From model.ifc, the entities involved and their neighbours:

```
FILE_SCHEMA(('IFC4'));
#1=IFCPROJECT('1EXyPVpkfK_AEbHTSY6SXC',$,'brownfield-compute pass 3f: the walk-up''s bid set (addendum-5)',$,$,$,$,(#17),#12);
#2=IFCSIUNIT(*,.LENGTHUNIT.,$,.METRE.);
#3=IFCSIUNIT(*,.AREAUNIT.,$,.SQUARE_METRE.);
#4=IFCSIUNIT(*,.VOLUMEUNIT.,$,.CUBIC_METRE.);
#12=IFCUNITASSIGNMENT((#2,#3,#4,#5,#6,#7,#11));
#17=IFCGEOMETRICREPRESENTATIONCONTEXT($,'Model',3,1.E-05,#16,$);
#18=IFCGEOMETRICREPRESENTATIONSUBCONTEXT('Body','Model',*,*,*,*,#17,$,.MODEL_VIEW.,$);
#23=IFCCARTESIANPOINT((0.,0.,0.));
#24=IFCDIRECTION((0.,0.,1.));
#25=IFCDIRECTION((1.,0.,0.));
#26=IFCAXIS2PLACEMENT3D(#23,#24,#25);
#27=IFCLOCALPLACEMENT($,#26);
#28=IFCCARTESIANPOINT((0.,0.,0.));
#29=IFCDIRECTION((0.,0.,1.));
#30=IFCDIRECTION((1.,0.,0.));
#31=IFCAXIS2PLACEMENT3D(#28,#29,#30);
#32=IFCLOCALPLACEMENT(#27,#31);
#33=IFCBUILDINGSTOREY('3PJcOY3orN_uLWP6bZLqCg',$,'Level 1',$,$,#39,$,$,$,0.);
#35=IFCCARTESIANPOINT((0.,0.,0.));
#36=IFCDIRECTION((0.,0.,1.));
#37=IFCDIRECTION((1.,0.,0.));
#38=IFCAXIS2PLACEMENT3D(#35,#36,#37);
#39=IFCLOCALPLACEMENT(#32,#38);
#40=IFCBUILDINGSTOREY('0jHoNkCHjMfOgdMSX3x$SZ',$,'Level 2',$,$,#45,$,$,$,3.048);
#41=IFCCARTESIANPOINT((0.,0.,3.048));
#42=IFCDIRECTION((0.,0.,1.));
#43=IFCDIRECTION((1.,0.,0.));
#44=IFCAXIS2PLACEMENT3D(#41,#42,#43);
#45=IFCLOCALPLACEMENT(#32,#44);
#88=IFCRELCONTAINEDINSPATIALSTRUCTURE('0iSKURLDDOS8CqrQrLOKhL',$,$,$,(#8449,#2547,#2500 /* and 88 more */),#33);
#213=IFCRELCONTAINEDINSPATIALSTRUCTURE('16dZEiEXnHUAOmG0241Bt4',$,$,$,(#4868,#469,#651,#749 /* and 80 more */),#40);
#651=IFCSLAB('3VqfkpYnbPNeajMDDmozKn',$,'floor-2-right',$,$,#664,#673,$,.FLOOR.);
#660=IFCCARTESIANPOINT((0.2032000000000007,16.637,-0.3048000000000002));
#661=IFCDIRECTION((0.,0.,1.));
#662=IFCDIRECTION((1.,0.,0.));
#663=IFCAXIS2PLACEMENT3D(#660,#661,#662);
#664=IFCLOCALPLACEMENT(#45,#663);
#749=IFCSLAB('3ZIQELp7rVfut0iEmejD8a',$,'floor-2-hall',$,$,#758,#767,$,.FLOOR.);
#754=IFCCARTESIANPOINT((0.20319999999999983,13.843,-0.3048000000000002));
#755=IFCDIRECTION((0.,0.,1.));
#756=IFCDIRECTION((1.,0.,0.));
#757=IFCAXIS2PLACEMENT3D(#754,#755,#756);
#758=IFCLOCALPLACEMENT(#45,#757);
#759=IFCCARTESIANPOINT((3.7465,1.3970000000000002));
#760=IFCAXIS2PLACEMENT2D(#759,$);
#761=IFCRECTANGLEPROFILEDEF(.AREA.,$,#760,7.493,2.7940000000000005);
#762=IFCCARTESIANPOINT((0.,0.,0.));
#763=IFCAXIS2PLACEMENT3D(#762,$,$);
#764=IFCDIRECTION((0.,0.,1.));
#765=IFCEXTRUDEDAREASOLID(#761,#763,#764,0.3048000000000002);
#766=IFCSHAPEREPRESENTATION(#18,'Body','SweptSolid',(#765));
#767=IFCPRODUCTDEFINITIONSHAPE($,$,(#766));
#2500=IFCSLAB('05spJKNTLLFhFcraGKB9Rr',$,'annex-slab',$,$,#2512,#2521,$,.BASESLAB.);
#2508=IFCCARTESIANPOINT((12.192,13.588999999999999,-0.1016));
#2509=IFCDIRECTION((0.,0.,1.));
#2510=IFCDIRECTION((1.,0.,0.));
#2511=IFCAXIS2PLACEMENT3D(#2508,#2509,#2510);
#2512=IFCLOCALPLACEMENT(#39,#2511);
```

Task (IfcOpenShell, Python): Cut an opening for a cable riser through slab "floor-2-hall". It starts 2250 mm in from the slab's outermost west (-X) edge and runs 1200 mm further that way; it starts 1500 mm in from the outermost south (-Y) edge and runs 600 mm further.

```python
import numpy as np
import ifcopenshell
import ifcopenshell.api.feature
import ifcopenshell.api.geometry
import ifcopenshell.api.root
import ifcopenshell.geom
import ifcopenshell.util.placement
import ifcopenshell.util.representation
import ifcopenshell.util.shape
import ifcopenshell.util.unit

model = ifcopenshell.open("model.ifc")
unit_scale = ifcopenshell.util.unit.calculate_unit_scale(model)
settings = ifcopenshell.geom.settings()


def volume(element):
    """Net volume in cubic metres, openings subtracted."""
    shape = ifcopenshell.geom.create_shape(settings, element)
    return ifcopenshell.util.shape.get_volume(shape.geometry)


slab = model.by_guid("3ZIQELp7rVfut0iEmejD8a")
before = volume(slab)

# Extent in the slab's own axes, in metres. The edges named are its -X and -Y sides.
slab_shape = ifcopenshell.geom.create_shape(settings, slab)
vertices = ifcopenshell.util.shape.get_vertices(slab_shape.geometry)
x_min, y_min, bottom = vertices.min(axis=0)
top = vertices[:, 2].max()

opening = ifcopenshell.api.root.create_entity(model, ifc_class="IfcOpeningElement", name="Cable riser opening", predefined_type="OPENING")
context = ifcopenshell.util.representation.get_context(model, "Model", "Body", "MODEL_VIEW")
width, depth = 1.2, 0.6
outline = [(0.0, 0.0), (width, 0.0), (width, depth), (0.0, depth), (0.0, 0.0)]
# Overshoot both faces by 50 mm so the cut is clean.
shape = ifcopenshell.api.geometry.add_slab_representation(
    model, context=context, depth=top - bottom + 0.1, polyline=outline
)
ifcopenshell.api.geometry.assign_representation(model, product=opening, representation=shape)

matrix = ifcopenshell.util.placement.get_local_placement(slab.ObjectPlacement)
matrix[:, 3] = matrix @ np.append(np.array([x_min + 2.25, y_min + 1.5, bottom - 0.05]) / unit_scale, 1.0)
ifcopenshell.api.geometry.edit_object_placement(model, product=opening, matrix=matrix, is_si=False)
ifcopenshell.api.feature.add_feature(model, feature=opening, element=slab)

after = volume(slab)

print(f"slab volume {before:.3f} -> {after:.3f} m3")

model.write("model_v2.ifc")
```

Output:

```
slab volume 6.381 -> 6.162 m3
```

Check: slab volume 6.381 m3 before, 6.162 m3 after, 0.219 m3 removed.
